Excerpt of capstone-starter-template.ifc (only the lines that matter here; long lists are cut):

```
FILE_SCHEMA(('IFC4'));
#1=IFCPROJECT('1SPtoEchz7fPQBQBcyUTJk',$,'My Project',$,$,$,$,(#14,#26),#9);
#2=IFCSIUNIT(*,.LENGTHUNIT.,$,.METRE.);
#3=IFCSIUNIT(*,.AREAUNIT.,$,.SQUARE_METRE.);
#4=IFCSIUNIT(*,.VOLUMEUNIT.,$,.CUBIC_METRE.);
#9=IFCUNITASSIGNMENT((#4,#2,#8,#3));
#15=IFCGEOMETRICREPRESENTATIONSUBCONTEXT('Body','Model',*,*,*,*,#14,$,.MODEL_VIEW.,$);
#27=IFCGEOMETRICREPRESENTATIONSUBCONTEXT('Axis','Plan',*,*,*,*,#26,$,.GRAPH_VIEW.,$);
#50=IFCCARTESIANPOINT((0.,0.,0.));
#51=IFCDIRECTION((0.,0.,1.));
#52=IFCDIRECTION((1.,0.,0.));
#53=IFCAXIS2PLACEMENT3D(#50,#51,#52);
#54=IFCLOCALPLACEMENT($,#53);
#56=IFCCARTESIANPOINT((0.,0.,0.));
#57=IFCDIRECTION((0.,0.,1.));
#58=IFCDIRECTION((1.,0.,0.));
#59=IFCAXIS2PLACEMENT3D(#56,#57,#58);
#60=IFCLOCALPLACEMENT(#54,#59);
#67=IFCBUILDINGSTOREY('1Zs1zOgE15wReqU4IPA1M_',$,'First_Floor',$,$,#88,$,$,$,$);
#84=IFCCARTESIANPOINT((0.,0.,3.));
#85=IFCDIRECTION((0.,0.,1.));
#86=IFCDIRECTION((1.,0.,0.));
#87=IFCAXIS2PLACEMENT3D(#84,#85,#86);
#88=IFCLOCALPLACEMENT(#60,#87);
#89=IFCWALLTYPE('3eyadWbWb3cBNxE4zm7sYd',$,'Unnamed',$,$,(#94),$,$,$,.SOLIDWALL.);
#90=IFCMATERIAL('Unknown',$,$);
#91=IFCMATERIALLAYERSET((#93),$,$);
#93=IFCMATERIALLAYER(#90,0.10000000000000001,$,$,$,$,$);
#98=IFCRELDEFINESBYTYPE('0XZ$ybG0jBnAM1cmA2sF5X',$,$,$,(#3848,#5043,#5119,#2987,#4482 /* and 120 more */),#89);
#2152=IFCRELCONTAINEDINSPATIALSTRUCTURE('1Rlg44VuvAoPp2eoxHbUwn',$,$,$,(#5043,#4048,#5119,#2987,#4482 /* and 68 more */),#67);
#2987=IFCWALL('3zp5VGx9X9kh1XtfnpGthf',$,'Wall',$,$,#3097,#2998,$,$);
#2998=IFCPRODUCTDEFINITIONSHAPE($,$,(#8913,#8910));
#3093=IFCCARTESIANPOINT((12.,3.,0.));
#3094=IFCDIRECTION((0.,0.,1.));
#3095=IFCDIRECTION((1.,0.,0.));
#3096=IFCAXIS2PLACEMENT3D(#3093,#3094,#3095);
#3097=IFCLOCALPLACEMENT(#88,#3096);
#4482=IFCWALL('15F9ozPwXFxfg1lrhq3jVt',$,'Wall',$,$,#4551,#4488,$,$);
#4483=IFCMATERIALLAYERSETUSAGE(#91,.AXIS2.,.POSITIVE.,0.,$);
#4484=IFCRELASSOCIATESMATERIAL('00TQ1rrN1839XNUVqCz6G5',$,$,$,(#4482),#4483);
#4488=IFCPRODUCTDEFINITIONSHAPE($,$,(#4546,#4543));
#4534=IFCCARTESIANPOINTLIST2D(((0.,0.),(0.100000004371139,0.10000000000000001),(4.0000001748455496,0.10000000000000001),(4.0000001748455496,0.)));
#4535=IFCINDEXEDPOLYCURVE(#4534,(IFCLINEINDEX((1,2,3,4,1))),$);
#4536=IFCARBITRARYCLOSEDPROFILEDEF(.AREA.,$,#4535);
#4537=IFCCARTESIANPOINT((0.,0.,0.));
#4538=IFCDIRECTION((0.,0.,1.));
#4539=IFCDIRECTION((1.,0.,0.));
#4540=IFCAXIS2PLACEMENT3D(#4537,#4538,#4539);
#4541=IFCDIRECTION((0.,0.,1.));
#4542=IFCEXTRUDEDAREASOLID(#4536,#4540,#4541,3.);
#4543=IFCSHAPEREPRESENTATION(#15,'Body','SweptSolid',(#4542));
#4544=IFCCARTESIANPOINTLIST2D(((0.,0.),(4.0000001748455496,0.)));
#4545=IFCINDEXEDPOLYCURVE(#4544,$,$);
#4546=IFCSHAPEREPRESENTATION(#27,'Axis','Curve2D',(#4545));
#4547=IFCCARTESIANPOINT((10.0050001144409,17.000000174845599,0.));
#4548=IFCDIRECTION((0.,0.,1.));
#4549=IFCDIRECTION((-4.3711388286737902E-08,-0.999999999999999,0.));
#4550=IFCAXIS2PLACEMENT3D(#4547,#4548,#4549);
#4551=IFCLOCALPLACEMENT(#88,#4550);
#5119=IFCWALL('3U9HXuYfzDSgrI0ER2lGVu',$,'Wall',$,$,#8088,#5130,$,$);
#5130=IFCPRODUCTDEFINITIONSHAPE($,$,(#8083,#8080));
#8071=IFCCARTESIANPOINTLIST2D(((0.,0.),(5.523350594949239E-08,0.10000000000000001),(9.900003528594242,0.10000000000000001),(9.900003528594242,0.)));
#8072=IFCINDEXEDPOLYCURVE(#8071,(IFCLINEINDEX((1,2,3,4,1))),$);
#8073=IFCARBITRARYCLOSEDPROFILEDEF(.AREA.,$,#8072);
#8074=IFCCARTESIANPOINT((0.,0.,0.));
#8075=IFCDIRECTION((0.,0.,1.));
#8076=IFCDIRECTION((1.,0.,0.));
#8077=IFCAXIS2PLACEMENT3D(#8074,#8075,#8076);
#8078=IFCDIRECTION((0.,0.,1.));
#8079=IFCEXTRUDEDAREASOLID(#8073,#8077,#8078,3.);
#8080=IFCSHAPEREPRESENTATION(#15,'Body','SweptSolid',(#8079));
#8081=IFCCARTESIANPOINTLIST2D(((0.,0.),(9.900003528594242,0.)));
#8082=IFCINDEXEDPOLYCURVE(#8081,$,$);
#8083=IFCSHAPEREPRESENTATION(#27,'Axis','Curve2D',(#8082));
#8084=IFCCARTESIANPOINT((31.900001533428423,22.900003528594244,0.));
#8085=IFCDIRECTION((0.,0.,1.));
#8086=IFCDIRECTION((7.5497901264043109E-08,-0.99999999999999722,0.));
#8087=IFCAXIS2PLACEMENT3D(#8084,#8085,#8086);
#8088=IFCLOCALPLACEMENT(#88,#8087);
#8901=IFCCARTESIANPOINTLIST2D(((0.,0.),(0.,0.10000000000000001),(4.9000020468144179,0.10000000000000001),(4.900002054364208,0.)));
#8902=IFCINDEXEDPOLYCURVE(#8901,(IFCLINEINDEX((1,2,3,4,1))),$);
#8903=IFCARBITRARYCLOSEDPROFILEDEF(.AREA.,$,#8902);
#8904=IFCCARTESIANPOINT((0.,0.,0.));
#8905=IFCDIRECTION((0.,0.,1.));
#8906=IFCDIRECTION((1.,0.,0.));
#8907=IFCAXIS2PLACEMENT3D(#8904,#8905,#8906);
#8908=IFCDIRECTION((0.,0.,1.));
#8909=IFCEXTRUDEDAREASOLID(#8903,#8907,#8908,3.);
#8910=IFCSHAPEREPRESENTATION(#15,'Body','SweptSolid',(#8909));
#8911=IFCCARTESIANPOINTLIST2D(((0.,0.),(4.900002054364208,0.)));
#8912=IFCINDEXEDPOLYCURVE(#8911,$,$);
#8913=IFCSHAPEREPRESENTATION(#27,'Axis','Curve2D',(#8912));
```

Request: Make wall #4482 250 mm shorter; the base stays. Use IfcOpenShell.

```python
import ifcopenshell
import ifcopenshell.geom
import ifcopenshell.util.representation
import ifcopenshell.util.shape
import ifcopenshell.util.unit

model = ifcopenshell.open("capstone-starter-template.ifc")
unit_scale = ifcopenshell.util.unit.calculate_unit_scale(model)
settings = ifcopenshell.geom.settings()


def volume(element):
    """Net volume in cubic metres, openings subtracted."""
    shape = ifcopenshell.geom.create_shape(settings, element)
    return ifcopenshell.util.shape.get_volume(shape.geometry)


wall = model.by_id(4482)
before = volume(wall)

body = ifcopenshell.util.representation.get_representation(wall, "Model", "Body")
solid = body.Items[0]
old_height = solid.Depth
solid.Depth -= 0.25 / unit_scale
after = volume(wall)

print(f"height {old_height:g} -> {solid.Depth:g}, volume {before:.3f} -> {after:.3f} m3")

model.write("capstone-starter-template-out.ifc")
```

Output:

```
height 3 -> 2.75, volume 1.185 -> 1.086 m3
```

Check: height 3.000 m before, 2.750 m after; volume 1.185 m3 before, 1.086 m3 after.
